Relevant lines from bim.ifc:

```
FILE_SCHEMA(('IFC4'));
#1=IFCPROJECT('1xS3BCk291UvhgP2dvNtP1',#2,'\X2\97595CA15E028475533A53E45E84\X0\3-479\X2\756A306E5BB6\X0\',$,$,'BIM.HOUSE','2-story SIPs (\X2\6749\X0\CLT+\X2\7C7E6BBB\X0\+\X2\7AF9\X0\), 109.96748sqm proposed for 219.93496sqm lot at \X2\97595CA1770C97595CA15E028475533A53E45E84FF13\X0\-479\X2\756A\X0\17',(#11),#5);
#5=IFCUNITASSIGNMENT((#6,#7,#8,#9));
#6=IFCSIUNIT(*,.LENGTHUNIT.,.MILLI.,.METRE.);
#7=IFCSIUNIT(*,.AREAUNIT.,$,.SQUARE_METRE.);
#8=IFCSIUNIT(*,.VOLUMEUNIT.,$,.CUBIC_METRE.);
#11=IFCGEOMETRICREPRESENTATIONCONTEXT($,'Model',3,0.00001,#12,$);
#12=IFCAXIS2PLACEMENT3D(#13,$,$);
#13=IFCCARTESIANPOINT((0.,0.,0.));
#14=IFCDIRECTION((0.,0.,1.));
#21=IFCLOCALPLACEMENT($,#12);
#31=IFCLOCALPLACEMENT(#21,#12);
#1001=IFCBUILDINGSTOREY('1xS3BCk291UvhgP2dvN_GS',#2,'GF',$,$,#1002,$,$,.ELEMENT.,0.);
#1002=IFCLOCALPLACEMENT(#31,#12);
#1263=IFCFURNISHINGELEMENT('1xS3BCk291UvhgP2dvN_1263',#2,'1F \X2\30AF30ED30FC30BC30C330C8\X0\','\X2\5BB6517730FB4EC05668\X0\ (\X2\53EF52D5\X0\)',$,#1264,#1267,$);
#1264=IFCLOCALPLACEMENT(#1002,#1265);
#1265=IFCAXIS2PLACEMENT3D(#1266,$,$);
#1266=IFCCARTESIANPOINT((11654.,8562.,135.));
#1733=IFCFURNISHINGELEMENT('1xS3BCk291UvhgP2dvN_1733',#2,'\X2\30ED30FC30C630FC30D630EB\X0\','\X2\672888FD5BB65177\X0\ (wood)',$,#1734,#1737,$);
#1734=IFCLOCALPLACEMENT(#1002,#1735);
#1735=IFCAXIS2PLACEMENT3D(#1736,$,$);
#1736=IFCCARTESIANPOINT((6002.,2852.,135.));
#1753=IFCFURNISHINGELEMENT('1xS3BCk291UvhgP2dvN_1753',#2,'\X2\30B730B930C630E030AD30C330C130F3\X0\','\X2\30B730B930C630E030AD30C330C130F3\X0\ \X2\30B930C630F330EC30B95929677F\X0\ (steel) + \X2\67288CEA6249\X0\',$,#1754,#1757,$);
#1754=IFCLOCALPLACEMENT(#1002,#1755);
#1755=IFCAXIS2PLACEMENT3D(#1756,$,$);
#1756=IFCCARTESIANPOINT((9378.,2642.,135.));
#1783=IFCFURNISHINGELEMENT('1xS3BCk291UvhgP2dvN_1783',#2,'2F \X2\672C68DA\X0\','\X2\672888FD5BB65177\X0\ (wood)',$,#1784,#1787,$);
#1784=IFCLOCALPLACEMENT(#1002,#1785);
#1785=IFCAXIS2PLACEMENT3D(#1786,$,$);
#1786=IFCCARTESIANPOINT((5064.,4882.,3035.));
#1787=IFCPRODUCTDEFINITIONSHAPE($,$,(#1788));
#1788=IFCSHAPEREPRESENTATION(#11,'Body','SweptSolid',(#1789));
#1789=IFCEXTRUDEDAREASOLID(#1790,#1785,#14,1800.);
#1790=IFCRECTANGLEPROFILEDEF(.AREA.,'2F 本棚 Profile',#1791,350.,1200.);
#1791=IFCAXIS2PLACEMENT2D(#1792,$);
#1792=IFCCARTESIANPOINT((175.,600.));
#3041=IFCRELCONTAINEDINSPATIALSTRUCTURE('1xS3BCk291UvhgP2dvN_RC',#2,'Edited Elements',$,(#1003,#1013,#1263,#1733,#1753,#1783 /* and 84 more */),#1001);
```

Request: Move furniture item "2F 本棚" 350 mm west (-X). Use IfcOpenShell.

```python
import ifcopenshell
import ifcopenshell.api.geometry
import ifcopenshell.util.placement
import ifcopenshell.util.unit

model = ifcopenshell.open("bim.ifc")
unit_scale = ifcopenshell.util.unit.calculate_unit_scale(model)

item = model.by_guid("1xS3BCk291UvhgP2dvN_1783")
matrix = ifcopenshell.util.placement.get_local_placement(item.ObjectPlacement)
matrix[0, 3] -= 0.35 / unit_scale
ifcopenshell.api.geometry.edit_object_placement(model, product=item, matrix=matrix, is_si=False)

print(ifcopenshell.util.placement.get_local_placement(item.ObjectPlacement).round(3) + 0.0)

model.write("bim_v2.ifc")
```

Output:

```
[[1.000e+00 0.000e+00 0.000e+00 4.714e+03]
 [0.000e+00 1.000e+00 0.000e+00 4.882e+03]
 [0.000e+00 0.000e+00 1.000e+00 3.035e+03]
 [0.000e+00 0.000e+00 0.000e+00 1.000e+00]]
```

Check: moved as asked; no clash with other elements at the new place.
